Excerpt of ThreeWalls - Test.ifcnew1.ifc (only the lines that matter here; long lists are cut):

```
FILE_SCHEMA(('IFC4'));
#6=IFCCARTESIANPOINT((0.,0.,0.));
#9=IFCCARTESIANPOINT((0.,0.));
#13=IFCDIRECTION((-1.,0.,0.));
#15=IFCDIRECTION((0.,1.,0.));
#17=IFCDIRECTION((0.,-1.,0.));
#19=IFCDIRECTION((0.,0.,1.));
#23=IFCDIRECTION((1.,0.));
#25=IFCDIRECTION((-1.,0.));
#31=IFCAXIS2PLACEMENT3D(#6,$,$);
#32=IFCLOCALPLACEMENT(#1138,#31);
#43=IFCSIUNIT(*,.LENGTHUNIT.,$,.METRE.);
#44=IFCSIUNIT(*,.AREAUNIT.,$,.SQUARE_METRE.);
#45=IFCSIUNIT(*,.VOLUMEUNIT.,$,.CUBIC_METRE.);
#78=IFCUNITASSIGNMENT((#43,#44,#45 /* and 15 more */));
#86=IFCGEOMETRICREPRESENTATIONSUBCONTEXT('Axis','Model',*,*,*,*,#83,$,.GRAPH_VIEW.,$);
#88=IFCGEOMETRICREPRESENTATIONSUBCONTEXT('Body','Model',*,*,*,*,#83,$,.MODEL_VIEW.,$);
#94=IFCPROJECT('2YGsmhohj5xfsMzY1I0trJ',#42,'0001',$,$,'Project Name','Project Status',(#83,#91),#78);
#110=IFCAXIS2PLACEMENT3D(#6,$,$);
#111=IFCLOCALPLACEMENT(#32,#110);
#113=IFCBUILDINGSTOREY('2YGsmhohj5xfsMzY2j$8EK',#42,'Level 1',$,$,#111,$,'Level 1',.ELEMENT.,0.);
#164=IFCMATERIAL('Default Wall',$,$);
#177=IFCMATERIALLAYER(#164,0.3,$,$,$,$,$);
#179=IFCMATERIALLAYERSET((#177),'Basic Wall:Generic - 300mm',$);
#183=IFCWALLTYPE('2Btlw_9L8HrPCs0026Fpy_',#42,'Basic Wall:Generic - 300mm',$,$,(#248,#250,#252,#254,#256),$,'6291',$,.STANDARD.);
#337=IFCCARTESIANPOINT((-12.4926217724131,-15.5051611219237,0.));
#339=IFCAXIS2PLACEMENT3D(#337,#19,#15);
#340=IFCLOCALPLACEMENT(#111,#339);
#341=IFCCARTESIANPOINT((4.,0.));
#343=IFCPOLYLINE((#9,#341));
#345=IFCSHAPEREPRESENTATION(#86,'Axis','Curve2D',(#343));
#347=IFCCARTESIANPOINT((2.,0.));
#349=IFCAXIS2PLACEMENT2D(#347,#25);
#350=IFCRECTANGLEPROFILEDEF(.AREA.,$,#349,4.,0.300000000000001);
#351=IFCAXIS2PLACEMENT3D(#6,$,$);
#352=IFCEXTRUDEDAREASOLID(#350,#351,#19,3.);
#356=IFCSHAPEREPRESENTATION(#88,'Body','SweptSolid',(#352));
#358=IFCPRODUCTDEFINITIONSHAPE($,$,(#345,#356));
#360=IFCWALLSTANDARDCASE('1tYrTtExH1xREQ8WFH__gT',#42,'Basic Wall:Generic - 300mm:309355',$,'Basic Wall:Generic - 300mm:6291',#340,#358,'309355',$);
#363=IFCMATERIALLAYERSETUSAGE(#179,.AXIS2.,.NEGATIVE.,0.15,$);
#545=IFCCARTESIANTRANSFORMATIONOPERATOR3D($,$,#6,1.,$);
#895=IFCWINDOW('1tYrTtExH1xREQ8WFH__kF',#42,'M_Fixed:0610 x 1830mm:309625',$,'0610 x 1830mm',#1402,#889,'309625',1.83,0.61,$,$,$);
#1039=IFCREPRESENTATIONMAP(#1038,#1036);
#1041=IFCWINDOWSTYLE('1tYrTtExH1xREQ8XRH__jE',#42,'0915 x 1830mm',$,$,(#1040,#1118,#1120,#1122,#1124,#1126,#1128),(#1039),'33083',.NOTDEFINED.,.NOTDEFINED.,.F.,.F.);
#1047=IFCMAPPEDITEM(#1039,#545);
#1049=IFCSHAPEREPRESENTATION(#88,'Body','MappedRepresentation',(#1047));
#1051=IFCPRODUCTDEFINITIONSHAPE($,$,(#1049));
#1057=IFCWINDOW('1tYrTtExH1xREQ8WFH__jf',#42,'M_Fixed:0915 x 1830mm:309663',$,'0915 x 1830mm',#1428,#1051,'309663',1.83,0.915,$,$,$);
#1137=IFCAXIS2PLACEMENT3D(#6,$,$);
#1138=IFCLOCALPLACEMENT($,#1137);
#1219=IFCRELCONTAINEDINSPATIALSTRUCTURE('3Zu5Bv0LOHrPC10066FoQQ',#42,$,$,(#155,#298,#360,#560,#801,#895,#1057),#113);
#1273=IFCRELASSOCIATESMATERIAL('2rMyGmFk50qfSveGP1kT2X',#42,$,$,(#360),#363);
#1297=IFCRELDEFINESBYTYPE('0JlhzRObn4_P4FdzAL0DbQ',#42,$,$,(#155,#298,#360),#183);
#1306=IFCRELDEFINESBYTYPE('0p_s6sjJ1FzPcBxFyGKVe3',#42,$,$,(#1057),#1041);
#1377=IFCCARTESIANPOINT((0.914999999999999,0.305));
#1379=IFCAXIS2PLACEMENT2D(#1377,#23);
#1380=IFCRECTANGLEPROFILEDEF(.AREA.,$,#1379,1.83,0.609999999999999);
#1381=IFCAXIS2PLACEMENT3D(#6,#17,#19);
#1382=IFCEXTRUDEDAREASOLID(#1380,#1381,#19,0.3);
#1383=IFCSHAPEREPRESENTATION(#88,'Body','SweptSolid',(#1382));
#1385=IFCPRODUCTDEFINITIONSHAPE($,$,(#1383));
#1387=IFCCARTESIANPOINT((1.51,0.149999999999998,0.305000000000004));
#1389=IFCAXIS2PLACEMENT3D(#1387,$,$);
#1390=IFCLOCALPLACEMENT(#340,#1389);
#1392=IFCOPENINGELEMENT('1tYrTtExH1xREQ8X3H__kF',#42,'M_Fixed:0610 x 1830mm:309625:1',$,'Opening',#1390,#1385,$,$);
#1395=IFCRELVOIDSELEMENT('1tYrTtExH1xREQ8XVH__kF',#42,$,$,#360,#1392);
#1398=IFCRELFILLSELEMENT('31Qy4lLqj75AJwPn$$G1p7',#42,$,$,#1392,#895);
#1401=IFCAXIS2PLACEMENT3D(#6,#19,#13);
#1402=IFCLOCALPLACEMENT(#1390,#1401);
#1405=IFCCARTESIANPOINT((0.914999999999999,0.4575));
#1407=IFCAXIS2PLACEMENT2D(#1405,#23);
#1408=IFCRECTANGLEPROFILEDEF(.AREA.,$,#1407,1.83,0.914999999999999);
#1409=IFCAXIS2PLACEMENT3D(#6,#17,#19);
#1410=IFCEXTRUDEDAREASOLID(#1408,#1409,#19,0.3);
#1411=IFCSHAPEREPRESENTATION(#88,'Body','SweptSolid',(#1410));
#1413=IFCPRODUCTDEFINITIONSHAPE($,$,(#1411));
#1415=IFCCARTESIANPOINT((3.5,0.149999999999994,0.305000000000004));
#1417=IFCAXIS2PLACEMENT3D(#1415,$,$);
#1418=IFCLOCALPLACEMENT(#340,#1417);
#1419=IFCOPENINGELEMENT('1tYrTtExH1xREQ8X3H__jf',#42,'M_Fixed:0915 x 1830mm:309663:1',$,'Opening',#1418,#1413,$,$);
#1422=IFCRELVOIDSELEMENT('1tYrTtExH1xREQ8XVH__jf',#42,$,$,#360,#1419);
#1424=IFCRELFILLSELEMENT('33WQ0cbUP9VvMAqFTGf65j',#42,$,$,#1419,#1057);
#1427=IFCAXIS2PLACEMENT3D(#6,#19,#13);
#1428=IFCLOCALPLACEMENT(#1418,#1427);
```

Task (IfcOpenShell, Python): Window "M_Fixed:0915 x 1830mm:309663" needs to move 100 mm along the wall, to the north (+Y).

```python
import ifcopenshell
import ifcopenshell.api.geometry
import ifcopenshell.util.placement

model = ifcopenshell.open("ThreeWalls - Test.ifcnew1.ifc")

window = model.by_guid("1tYrTtExH1xREQ8WFH__jf")
opening = window.FillsVoids[0].RelatingOpeningElement
wall = opening.VoidsElements[0].RelatingBuildingElement

wall_matrix = ifcopenshell.util.placement.get_local_placement(wall.ObjectPlacement)
shift = wall_matrix[:3, 0] * 0.1
before = ifcopenshell.util.placement.get_local_placement(window.ObjectPlacement)[:3, 3].copy()

# The window is placed relative to its opening, so it follows when the opening moves.
matrix = ifcopenshell.util.placement.get_local_placement(opening.ObjectPlacement)
matrix[:3, 3] += shift
ifcopenshell.api.geometry.edit_object_placement(
    model, product=opening, matrix=matrix, is_si=False, should_transform_children=True
)

after = ifcopenshell.util.placement.get_local_placement(window.ObjectPlacement)[:3, 3]
print("window moved by", (after - before).round(3) + 0.0)

model.write("ThreeWalls - Test.ifcnew1_edited.ifc")
```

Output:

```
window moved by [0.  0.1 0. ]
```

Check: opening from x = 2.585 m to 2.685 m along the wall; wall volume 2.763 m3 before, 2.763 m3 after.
